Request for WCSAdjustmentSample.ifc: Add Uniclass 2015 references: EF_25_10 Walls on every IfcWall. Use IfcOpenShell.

First a look at what the model holds.

```python
import ifcopenshell

model = ifcopenshell.open("WCSAdjustmentSample.ifc")
print(model.schema)
print("classifications:", [c.Name for c in model.by_type("IfcClassification")])
for ifc_class in ("IfcDoor", "IfcRoof", "IfcStair", "IfcWall", "IfcWindow"):
    print(ifc_class, len(model.by_type(ifc_class)))
```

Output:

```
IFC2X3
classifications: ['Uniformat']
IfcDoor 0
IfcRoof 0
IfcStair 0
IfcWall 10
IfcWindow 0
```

```python
import ifcopenshell
import ifcopenshell.api.classification

model = ifcopenshell.open("WCSAdjustmentSample.ifc")

# IFC2X3 requires Source and Edition and has no link from the project to the system.
system = model.create_entity("IfcClassification", Source="NBS", Edition="2015", Name="Uniclass 2015")

codes = {
    "IfcWall": ("EF_25_10", "Walls"),
}
for ifc_class, (code, name) in codes.items():
    products = model.by_type(ifc_class)
    ifcopenshell.api.classification.add_reference(
        model, products=products, classification=system, identification=code, name=name
    )
    print(code, len(products))

model.write("WCSAdjustmentSample_edited.ifc")
```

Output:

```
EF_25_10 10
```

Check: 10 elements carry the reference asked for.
